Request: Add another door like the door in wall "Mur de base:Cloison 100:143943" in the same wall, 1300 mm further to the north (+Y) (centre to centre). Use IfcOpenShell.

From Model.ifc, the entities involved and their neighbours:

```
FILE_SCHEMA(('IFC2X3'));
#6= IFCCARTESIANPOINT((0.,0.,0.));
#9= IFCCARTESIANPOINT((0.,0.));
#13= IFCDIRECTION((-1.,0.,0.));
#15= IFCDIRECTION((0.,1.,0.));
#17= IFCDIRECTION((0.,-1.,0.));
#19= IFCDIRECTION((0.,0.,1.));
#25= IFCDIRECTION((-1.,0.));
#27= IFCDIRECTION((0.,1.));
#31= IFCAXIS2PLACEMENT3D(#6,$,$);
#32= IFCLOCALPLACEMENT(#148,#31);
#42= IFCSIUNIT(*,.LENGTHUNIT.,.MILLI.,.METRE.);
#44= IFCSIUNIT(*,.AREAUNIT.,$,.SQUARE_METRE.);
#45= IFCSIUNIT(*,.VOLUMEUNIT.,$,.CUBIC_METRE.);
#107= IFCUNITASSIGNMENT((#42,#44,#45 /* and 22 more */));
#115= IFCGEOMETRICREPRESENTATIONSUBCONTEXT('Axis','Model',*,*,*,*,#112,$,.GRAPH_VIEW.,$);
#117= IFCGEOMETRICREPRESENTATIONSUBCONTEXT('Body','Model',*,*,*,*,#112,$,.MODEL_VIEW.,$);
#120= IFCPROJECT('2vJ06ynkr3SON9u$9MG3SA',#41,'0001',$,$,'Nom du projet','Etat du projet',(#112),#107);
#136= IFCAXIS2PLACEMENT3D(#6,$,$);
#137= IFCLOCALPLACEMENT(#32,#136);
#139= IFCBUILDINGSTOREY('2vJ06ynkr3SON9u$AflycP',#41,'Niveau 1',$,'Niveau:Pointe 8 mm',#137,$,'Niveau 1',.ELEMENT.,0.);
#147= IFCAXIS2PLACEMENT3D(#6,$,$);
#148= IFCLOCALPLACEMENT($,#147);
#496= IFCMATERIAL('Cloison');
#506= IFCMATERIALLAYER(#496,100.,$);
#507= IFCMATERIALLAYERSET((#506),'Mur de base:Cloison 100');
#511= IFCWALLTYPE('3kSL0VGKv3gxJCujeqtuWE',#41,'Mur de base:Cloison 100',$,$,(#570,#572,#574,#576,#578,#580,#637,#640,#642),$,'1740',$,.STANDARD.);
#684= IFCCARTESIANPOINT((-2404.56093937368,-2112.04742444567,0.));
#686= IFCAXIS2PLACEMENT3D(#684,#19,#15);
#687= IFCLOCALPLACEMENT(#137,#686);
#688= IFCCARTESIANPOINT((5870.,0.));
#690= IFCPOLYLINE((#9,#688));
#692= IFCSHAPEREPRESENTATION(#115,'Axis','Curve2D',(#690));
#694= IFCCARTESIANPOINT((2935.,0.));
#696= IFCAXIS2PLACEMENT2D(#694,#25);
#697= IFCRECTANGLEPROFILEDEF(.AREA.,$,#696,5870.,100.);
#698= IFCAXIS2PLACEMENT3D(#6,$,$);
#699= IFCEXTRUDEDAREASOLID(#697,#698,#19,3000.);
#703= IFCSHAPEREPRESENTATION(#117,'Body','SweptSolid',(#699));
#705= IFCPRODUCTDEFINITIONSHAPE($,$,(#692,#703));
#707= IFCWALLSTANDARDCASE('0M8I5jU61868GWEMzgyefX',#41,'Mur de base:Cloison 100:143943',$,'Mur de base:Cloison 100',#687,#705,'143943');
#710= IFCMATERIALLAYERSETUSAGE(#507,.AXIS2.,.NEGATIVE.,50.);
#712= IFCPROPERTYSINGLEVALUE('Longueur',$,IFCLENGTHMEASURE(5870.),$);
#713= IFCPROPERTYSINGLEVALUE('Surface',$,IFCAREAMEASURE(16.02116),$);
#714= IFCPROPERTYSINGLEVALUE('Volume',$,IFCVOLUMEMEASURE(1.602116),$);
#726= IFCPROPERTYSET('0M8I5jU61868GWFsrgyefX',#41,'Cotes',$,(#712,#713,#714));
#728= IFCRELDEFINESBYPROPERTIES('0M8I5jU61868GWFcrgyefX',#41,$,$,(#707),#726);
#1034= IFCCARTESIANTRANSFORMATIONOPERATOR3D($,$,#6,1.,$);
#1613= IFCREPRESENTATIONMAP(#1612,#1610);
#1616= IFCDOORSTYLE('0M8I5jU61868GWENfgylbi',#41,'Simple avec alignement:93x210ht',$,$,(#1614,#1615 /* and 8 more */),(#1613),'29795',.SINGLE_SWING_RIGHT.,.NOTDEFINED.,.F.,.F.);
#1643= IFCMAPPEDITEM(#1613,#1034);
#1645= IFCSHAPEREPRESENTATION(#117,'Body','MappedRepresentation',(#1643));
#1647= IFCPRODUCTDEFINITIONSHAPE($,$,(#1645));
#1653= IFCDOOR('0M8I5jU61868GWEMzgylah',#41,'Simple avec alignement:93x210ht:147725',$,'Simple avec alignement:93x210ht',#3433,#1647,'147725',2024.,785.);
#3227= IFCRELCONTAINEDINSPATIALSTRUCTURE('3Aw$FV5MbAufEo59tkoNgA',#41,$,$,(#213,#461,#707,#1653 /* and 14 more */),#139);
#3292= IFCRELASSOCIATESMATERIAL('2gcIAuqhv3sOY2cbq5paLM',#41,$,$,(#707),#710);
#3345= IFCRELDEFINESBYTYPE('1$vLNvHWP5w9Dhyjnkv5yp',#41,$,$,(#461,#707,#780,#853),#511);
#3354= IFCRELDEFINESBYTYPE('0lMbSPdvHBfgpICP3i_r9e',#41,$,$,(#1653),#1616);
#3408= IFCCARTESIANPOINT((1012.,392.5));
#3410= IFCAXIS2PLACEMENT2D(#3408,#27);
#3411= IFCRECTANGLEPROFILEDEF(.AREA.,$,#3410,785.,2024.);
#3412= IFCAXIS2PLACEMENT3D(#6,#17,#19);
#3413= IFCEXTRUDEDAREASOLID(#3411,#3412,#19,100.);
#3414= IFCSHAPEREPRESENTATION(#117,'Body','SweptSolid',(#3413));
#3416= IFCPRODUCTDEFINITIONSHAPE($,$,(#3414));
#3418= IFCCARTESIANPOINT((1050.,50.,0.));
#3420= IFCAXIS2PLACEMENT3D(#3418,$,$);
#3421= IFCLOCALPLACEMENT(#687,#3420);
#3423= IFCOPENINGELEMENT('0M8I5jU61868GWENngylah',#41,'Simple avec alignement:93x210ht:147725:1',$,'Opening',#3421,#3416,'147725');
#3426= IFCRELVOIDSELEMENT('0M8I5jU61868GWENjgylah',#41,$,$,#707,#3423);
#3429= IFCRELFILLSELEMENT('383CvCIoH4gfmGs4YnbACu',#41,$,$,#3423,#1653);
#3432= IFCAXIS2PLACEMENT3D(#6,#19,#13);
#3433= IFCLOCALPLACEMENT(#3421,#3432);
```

```python
import ifcopenshell
import ifcopenshell.api.feature
import ifcopenshell.api.geometry
import ifcopenshell.api.pset
import ifcopenshell.api.root
import ifcopenshell.geom
import ifcopenshell.util.element
import ifcopenshell.util.placement
import ifcopenshell.util.shape
import ifcopenshell.util.unit

model = ifcopenshell.open("Model.ifc")
unit_scale = ifcopenshell.util.unit.calculate_unit_scale(model)
area_scale = ifcopenshell.util.unit.calculate_unit_scale(model, "AREAUNIT")
volume_scale = ifcopenshell.util.unit.calculate_unit_scale(model, "VOLUMEUNIT")
settings = ifcopenshell.geom.settings()


def volume(element):
    """Net volume in cubic metres, openings subtracted."""
    shape = ifcopenshell.geom.create_shape(settings, element)
    return ifcopenshell.util.shape.get_volume(shape.geometry)


def reuse_history(source, copy):
    """copy_class also copies each property set's owner history, people and application; keep the originals."""
    for rel in copy.IsDefinedBy:
        if rel.is_a("IfcRelDefinesByProperties") and (history := rel.RelatingPropertyDefinition.OwnerHistory):
            rel.RelatingPropertyDefinition.OwnerHistory = source.OwnerHistory
            ifcopenshell.util.element.remove_deep2(model, history)


door = model.by_guid("0M8I5jU61868GWEMzgylah")
opening = door.FillsVoids[0].RelatingOpeningElement
wall = opening.VoidsElements[0].RelatingBuildingElement
before = volume(wall)
shift = ifcopenshell.util.placement.get_local_placement(wall.ObjectPlacement)[:3, 0] * 1.3 / unit_scale

# copy_class copies the void relationship, type, container and properties, but no geometry.
new_opening = ifcopenshell.api.root.copy_class(model, product=opening)
new_opening.Representation = ifcopenshell.util.element.copy_deep(
    model, opening.Representation, exclude=["IfcGeometricRepresentationContext", "IfcRepresentationMap"]
)
new_opening.Name = "Simple avec alignement:93x210ht"
new_opening.Tag = None
new_door = ifcopenshell.api.root.copy_class(model, product=door)
new_door.Representation = ifcopenshell.util.element.copy_deep(
    model, door.Representation, exclude=["IfcGeometricRepresentationContext", "IfcRepresentationMap"]
)
new_door.Name = "Simple avec alignement:93x210ht"
new_door.Tag = None
reuse_history(door, new_door)
fills = ifcopenshell.api.feature.add_filling(model, opening=new_opening, element=new_door)
fills.OwnerHistory = new_door.OwnerHistory  # required in IFC2X3

for old, new in ((opening, new_opening), (door, new_door)):
    matrix = ifcopenshell.util.placement.get_local_placement(old.ObjectPlacement)
    matrix[:3, 3] += shift
    ifcopenshell.api.geometry.edit_object_placement(model, product=new, matrix=matrix, is_si=False)

after = volume(wall)
thickness = 0.1  # wall thickness in metres

# Update the wall's stored quantities.
pset = model.by_id(ifcopenshell.util.element.get_pset(wall, "Cotes", should_inherit=False)["id"])
ifcopenshell.api.pset.edit_pset(model, pset=pset, properties={
    "Surface": model.create_entity("IfcAreaMeasure", after / thickness / area_scale),
    "Volume": model.create_entity("IfcVolumeMeasure", after / volume_scale),
})

print(f"wall volume {before:.3f} -> {after:.3f} m3")

model.write("Model_edited.ifc")
```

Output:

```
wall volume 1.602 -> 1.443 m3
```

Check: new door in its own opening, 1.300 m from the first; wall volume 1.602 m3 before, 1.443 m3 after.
